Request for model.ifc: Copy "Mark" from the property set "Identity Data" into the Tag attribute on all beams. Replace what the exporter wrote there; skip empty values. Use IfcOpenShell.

First a look at what the model holds.

```python
import ifcopenshell
import ifcopenshell.util.element

model = ifcopenshell.open("model.ifc")
print(model.schema)
beams = model.by_type("IfcBeam")
print(len(beams), "beams")
for e in beams[:8]:
    source = ifcopenshell.util.element.get_pset(e, "Identity Data", "Mark")
    target = e.Tag
    print(e.id(), repr(source), repr(target), sep=" | ")
```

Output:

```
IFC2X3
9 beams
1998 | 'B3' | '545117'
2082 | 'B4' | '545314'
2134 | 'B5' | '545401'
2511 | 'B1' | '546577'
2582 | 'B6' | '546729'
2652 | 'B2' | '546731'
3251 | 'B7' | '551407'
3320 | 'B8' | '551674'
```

```python
import ifcopenshell
import ifcopenshell.util.element

model = ifcopenshell.open("model.ifc")

count = 0
for e in model.by_type("IfcBeam"):
    value = ifcopenshell.util.element.get_pset(e, "Identity Data", "Mark")
    current = e.Tag
    if not value or not value.strip() or current == value:
        continue
    e.Tag = value
    count += 1

print(count, "beams updated")

model.write("model_v2.ifc")
```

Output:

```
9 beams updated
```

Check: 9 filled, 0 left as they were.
